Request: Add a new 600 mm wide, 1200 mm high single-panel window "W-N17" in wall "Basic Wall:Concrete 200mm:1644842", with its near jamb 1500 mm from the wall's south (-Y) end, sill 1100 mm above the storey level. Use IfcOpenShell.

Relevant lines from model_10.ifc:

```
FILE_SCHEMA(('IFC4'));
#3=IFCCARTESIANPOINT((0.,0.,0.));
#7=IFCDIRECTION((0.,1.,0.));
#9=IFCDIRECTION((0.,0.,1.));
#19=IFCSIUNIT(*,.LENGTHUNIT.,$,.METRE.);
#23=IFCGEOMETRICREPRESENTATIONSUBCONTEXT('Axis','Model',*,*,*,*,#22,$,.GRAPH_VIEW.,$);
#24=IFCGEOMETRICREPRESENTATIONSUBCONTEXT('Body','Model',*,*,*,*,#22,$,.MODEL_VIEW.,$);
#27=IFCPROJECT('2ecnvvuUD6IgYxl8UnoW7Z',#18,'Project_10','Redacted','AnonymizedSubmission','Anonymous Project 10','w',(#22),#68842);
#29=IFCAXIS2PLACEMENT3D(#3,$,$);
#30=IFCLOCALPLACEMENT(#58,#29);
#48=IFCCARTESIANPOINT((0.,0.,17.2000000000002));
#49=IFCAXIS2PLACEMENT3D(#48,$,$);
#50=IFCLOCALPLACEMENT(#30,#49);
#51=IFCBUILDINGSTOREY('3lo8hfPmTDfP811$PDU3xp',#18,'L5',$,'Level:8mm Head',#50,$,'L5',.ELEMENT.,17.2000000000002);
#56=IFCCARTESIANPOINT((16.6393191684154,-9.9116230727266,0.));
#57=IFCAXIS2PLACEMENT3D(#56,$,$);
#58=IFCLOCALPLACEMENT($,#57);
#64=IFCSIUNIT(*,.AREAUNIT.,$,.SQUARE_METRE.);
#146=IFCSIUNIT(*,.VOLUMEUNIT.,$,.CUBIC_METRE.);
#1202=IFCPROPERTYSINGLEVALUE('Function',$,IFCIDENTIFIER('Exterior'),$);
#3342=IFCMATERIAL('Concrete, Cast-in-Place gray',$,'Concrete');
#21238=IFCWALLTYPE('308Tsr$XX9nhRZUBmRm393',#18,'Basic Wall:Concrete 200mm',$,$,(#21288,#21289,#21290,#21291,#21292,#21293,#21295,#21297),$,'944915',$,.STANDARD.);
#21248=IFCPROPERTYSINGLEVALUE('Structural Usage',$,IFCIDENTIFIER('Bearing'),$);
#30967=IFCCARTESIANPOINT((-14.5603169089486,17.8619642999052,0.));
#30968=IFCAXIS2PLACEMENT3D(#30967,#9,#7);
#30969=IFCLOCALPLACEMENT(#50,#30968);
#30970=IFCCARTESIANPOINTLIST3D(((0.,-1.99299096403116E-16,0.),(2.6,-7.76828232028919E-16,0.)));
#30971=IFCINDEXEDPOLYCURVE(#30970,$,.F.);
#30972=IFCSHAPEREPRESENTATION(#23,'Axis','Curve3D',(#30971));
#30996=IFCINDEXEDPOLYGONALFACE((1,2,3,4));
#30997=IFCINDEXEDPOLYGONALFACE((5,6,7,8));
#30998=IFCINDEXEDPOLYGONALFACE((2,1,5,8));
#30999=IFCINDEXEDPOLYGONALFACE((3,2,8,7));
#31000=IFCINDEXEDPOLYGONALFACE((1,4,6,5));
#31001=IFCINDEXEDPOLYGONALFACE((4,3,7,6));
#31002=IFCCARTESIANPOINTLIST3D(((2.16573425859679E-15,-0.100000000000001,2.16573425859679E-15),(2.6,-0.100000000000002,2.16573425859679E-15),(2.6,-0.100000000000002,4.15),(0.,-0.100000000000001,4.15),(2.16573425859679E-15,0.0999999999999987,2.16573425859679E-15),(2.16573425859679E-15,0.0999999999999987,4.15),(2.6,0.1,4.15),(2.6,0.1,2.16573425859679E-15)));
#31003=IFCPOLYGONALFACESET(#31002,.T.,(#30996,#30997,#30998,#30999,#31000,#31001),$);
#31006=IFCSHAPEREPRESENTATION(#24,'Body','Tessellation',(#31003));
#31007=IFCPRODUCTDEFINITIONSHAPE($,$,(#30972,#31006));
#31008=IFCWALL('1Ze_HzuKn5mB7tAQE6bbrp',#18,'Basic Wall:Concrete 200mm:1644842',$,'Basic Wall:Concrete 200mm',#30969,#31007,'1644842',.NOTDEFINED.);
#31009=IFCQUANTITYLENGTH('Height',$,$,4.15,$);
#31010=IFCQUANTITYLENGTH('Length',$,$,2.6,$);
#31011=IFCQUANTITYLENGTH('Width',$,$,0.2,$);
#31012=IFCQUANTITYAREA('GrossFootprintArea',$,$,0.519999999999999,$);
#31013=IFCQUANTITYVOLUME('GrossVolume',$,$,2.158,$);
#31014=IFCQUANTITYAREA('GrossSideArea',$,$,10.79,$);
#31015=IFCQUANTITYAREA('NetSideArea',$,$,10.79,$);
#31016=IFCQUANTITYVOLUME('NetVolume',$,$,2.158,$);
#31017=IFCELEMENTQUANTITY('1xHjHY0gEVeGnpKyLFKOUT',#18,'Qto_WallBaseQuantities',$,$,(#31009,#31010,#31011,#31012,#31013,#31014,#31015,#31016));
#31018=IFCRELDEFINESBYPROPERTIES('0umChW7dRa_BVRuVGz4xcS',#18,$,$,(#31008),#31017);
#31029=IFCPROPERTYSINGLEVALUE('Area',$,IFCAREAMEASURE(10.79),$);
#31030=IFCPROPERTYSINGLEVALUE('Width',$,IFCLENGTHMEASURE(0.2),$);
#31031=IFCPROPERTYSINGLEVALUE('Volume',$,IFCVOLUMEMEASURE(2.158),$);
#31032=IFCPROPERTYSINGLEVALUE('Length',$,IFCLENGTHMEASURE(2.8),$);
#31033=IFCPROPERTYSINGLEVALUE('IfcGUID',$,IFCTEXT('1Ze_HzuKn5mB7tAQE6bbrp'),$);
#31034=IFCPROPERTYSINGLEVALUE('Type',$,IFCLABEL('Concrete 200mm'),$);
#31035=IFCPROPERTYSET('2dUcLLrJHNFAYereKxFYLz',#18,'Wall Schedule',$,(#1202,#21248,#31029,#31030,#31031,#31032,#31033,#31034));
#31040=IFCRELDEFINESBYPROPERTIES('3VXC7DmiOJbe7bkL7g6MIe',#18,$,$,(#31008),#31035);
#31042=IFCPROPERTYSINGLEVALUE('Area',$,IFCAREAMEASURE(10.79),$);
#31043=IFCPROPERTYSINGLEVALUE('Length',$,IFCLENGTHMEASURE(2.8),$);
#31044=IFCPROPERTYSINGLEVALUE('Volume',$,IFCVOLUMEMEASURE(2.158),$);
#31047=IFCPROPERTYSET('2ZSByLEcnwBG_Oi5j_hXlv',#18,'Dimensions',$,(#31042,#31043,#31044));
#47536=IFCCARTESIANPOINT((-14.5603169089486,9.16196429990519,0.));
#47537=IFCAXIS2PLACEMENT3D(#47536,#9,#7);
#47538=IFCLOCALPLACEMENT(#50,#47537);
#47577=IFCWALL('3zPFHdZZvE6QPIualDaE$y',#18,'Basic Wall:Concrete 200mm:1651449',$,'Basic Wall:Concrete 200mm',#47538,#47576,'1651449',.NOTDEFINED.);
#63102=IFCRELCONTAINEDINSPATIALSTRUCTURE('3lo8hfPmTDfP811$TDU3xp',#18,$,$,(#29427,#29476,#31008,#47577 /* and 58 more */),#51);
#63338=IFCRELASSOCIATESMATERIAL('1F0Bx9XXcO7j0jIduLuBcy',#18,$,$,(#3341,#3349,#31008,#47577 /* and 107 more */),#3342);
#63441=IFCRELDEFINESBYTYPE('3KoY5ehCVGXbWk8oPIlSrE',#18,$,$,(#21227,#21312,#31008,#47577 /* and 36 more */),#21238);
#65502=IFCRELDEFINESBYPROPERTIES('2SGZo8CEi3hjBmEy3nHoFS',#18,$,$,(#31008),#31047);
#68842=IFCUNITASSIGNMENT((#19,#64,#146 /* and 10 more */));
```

```python
import numpy as np
import ifcopenshell
import ifcopenshell.api.feature
import ifcopenshell.api.geometry
import ifcopenshell.api.pset
import ifcopenshell.api.root
import ifcopenshell.api.spatial
import ifcopenshell.geom
import ifcopenshell.util.element
import ifcopenshell.util.placement
import ifcopenshell.util.representation
import ifcopenshell.util.shape
import ifcopenshell.util.unit

model = ifcopenshell.open("model_10.ifc")
unit_scale = ifcopenshell.util.unit.calculate_unit_scale(model)
area_scale = ifcopenshell.util.unit.calculate_unit_scale(model, "AREAUNIT")
volume_scale = ifcopenshell.util.unit.calculate_unit_scale(model, "VOLUMEUNIT")
settings = ifcopenshell.geom.settings()


def volume(element):
    """Net volume in cubic metres, openings subtracted."""
    shape = ifcopenshell.geom.create_shape(settings, element)
    return ifcopenshell.util.shape.get_volume(shape.geometry)


wall = model.by_id(31008)
storey = ifcopenshell.util.element.get_container(wall, ifc_class="IfcBuildingStorey")
context = ifcopenshell.util.representation.get_context(model, "Model", "Body", "MODEL_VIEW")
before = volume(wall)

width, height, from_end, sill = 0.6, 1.2, 1.5, 1.1  # metres

# The wall runs along its own X axis, and the end named is its -X end.
wall_shape = ifcopenshell.geom.create_shape(settings, wall)
x, y, z = ifcopenshell.util.shape.get_vertices(wall_shape.geometry).T
start = x.min() + from_end
face, thickness = float(y.min()), float(y.max() - y.min())
wall_matrix = ifcopenshell.util.placement.get_local_placement(wall.ObjectPlacement)
level = ifcopenshell.util.placement.get_local_placement(storey.ObjectPlacement)[2, 3]


def in_wall(x, y):
    """Placement at x, y metres in the wall's axes, at sill height."""
    matrix = wall_matrix.copy()
    matrix[:, 3] = wall_matrix @ np.array([x / unit_scale, y / unit_scale, 0.0, 1.0])
    matrix[2, 3] = level + sill / unit_scale
    return matrix


# Opening: a box that overshoots both wall faces by 50 mm.
opening = ifcopenshell.api.root.create_entity(model, ifc_class="IfcOpeningElement", predefined_type="OPENING")
box = ifcopenshell.api.geometry.add_wall_representation(
    model, context=context, length=width, height=height, thickness=thickness + 0.1
)
ifcopenshell.api.geometry.assign_representation(model, product=opening, representation=box)
ifcopenshell.api.geometry.edit_object_placement(model, product=opening, matrix=in_wall(start, face - 0.05), is_si=False)
ifcopenshell.api.feature.add_feature(model, feature=opening, element=wall)

window = ifcopenshell.api.root.create_entity(model, ifc_class="IfcWindow", name="W-N17", predefined_type="WINDOW")
window.OverallWidth, window.OverallHeight = width / unit_scale, height / unit_scale
window.PartitioningType = "SINGLE_PANEL"
body = ifcopenshell.api.geometry.add_window_representation(
    model,
    context=context,
    overall_width=window.OverallWidth,
    overall_height=window.OverallHeight,
    partition_type="SINGLE_PANEL",
)
ifcopenshell.api.geometry.assign_representation(model, product=window, representation=body)
ifcopenshell.api.spatial.assign_container(model, products=[window], relating_structure=storey)
ifcopenshell.api.feature.add_filling(model, opening=opening, element=window)

# Centre the window in the wall's thickness.
ifcopenshell.api.geometry.edit_object_placement(model, product=window, matrix=in_wall(start, face), is_si=False)
window_shape = ifcopenshell.geom.create_shape(settings, window)
depth = ifcopenshell.util.shape.get_vertices(window_shape.geometry)[:, 1]
offset = face + thickness / 2 - (depth.min() + depth.max()) / 2
ifcopenshell.api.geometry.edit_object_placement(model, product=window, matrix=in_wall(start, offset), is_si=False)

after = volume(wall)

# Update the wall's stored quantities.
qto = model.by_id(ifcopenshell.util.element.get_pset(wall, "Qto_WallBaseQuantities", should_inherit=False)["id"])
ifcopenshell.api.pset.edit_qto(model, qto=qto, properties={
    "NetSideArea": after / thickness / area_scale,
    "NetVolume": after / volume_scale,
})
pset = model.by_id(ifcopenshell.util.element.get_pset(wall, "Wall Schedule", should_inherit=False)["id"])
ifcopenshell.api.pset.edit_pset(model, pset=pset, properties={
    "Area": model.create_entity("IfcAreaMeasure", after / thickness / area_scale),
    "Volume": model.create_entity("IfcVolumeMeasure", after / volume_scale),
})
pset = model.by_id(ifcopenshell.util.element.get_pset(wall, "Dimensions", should_inherit=False)["id"])
ifcopenshell.api.pset.edit_pset(model, pset=pset, properties={
    "Area": model.create_entity("IfcAreaMeasure", after / thickness / area_scale),
    "Volume": model.create_entity("IfcVolumeMeasure", after / volume_scale),
})

print(f"wall volume {before:.3f} -> {after:.3f} m3")

model.write("model_10_edited.ifc")
```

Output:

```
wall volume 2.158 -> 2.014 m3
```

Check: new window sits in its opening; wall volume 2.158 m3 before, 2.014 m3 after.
